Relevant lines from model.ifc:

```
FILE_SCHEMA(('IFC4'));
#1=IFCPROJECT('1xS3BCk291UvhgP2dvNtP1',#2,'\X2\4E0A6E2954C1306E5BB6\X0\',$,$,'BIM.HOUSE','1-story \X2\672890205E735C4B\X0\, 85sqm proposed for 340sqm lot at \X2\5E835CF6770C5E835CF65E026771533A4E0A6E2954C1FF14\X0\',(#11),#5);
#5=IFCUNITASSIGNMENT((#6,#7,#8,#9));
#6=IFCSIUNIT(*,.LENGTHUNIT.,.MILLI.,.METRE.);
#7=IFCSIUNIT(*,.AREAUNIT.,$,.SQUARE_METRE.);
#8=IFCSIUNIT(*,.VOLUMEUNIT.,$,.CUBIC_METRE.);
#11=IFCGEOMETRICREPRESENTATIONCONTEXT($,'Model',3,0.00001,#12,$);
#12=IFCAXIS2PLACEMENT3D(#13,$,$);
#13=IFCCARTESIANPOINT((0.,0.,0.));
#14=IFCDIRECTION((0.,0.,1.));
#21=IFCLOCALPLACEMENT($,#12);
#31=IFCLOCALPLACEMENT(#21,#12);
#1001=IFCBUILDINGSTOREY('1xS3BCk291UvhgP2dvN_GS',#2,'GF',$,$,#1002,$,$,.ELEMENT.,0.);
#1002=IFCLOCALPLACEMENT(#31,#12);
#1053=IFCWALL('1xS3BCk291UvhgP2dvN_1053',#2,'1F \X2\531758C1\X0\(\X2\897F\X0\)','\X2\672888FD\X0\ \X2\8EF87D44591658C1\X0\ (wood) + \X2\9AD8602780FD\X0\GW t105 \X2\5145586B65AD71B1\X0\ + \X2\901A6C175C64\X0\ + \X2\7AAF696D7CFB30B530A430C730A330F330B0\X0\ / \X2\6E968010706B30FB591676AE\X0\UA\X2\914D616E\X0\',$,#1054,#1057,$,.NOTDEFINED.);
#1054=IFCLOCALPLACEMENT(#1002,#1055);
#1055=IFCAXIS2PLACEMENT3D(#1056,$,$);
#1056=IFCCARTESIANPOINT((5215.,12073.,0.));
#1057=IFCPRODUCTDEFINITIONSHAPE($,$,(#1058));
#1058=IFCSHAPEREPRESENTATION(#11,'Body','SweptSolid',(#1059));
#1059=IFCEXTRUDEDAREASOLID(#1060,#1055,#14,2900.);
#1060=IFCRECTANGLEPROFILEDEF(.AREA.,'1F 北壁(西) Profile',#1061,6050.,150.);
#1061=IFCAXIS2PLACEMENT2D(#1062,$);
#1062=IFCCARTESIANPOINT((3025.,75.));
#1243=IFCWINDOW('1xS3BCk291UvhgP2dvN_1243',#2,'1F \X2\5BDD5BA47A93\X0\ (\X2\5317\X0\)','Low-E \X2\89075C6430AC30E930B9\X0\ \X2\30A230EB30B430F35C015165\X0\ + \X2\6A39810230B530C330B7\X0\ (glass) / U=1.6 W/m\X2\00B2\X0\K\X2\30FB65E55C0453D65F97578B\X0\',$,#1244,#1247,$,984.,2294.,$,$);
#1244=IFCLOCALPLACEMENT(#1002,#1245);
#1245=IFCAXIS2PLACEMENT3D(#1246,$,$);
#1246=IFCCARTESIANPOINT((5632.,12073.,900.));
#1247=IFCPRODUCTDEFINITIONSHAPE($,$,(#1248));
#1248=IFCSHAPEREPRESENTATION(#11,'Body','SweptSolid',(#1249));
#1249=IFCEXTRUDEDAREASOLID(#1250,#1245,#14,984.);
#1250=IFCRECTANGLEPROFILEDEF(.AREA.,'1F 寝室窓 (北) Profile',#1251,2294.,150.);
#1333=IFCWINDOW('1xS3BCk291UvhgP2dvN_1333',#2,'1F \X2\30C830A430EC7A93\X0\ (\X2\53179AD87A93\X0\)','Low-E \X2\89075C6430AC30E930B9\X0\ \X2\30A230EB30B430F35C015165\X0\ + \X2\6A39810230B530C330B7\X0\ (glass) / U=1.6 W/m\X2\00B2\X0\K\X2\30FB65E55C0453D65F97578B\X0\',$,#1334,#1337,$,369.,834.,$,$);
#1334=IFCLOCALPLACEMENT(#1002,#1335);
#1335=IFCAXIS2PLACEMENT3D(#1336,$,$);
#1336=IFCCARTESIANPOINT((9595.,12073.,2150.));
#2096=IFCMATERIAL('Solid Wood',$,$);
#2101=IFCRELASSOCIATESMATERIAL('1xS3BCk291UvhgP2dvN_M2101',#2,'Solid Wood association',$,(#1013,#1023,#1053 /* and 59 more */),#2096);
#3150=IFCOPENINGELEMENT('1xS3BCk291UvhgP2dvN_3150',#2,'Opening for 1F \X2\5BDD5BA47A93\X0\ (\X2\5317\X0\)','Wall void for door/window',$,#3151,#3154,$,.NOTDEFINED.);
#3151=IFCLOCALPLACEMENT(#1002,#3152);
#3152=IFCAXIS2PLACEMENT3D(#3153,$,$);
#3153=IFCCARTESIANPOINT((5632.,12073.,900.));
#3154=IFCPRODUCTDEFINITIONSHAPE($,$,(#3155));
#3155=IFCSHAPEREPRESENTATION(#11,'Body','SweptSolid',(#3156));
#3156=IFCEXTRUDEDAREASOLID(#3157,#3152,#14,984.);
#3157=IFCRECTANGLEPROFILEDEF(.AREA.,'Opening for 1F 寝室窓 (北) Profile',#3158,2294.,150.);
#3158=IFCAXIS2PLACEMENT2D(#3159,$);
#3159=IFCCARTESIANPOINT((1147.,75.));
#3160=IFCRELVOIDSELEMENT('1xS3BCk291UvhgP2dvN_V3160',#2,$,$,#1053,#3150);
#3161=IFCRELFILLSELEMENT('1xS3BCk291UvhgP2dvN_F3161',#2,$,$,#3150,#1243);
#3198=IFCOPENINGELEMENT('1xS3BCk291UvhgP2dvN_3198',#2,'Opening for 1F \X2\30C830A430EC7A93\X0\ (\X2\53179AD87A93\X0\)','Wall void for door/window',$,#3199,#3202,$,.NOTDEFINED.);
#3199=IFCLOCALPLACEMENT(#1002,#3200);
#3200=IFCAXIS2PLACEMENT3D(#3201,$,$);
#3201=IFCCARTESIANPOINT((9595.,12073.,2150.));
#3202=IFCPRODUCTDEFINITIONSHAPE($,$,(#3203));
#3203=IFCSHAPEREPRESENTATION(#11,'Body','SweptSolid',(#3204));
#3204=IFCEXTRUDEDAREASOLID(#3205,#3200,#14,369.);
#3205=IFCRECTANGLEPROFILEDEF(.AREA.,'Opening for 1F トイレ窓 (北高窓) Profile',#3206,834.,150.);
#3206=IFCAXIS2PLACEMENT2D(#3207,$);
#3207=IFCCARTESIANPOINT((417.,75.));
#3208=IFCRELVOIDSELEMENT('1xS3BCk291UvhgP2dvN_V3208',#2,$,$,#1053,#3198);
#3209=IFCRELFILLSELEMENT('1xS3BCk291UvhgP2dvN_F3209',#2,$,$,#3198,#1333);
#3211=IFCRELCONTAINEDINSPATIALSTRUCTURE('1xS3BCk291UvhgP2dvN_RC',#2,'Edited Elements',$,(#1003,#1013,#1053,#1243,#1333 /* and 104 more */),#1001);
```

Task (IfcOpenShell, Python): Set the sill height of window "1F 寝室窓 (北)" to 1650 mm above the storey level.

```python
import numpy as np
import ifcopenshell
import ifcopenshell.api.geometry
import ifcopenshell.geom
import ifcopenshell.util.element
import ifcopenshell.util.placement
import ifcopenshell.util.shape
import ifcopenshell.util.unit

model = ifcopenshell.open("model.ifc")
unit_scale = ifcopenshell.util.unit.calculate_unit_scale(model)

window = model.by_id(1243)
opening = window.FillsVoids[0].RelatingOpeningElement
storey = ifcopenshell.util.element.get_container(window, ifc_class="IfcBuildingStorey")
level = ifcopenshell.util.placement.get_local_placement(storey.ObjectPlacement)[2, 3]

# The opening's origin need not be at the sill, so measure its lowest point.
shape = ifcopenshell.geom.create_shape(ifcopenshell.geom.settings(), opening)
bottom = ifcopenshell.util.shape.get_shape_bottom_elevation(shape, shape.geometry) / unit_scale
dz = level + 1650.0 - bottom

shift = np.array([0.0, 0.0, dz])
# The window is not placed relative to its opening, so move both.
for product in (opening, window):
    matrix = ifcopenshell.util.placement.get_local_placement(product.ObjectPlacement)
    matrix[:3, 3] += shift
    ifcopenshell.api.geometry.edit_object_placement(model, product=product, matrix=matrix, is_si=False)

print(f"moved by {dz * unit_scale:+.3f} m")

model.write("model_rev.ifc")
```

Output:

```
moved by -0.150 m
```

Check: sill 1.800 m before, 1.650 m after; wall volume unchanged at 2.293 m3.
